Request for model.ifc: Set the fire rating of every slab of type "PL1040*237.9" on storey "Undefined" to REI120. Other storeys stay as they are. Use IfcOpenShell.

First a look at what the model holds.

```python
import ifcopenshell
import ifcopenshell.util.element

model = ifcopenshell.open("model.ifc")
print(model.schema)
storey = next(s for s in model.by_type("IfcBuildingStorey") if s.Name == "Undefined")
slabs = [e for e in ifcopenshell.util.element.get_decomposition(storey) if e.is_a("IfcSlab")]
seen = {}
for e in slabs:
    element_type = ifcopenshell.util.element.get_type(e)
    key = (element_type.Name if element_type != e and element_type else None, ifcopenshell.util.element.get_pset(e, "Pset_SlabCommon", "FireRating"))
    seen[key] = seen.get(key, 0) + 1
for (name, value), count in sorted(seen.items(), key=str):
    print(count, "x", name, "|", value)
```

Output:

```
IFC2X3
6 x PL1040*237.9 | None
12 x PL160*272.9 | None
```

```python
import ifcopenshell
import ifcopenshell.api.pset
import ifcopenshell.util.element

model = ifcopenshell.open("model.ifc")

storey = next(s for s in model.by_type("IfcBuildingStorey") if s.Name == "Undefined")
slabs = [e for e in ifcopenshell.util.element.get_decomposition(storey) if e.is_a("IfcSlab")]

count = 0
for e in slabs:
    element_type = ifcopenshell.util.element.get_type(e)
    if element_type in (None, e) or element_type.Name != "PL1040*237.9":
        continue
    # add_pset returns the element's existing set when there is one.
    pset = ifcopenshell.api.pset.add_pset(model, product=e, name="Pset_SlabCommon")
    ifcopenshell.api.pset.edit_pset(model, pset=pset, properties={"FireRating": "REI120"})
    count += 1

print(count, "slabs updated")

model.write("model_v2.ifc")
```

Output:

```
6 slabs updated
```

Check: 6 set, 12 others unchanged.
